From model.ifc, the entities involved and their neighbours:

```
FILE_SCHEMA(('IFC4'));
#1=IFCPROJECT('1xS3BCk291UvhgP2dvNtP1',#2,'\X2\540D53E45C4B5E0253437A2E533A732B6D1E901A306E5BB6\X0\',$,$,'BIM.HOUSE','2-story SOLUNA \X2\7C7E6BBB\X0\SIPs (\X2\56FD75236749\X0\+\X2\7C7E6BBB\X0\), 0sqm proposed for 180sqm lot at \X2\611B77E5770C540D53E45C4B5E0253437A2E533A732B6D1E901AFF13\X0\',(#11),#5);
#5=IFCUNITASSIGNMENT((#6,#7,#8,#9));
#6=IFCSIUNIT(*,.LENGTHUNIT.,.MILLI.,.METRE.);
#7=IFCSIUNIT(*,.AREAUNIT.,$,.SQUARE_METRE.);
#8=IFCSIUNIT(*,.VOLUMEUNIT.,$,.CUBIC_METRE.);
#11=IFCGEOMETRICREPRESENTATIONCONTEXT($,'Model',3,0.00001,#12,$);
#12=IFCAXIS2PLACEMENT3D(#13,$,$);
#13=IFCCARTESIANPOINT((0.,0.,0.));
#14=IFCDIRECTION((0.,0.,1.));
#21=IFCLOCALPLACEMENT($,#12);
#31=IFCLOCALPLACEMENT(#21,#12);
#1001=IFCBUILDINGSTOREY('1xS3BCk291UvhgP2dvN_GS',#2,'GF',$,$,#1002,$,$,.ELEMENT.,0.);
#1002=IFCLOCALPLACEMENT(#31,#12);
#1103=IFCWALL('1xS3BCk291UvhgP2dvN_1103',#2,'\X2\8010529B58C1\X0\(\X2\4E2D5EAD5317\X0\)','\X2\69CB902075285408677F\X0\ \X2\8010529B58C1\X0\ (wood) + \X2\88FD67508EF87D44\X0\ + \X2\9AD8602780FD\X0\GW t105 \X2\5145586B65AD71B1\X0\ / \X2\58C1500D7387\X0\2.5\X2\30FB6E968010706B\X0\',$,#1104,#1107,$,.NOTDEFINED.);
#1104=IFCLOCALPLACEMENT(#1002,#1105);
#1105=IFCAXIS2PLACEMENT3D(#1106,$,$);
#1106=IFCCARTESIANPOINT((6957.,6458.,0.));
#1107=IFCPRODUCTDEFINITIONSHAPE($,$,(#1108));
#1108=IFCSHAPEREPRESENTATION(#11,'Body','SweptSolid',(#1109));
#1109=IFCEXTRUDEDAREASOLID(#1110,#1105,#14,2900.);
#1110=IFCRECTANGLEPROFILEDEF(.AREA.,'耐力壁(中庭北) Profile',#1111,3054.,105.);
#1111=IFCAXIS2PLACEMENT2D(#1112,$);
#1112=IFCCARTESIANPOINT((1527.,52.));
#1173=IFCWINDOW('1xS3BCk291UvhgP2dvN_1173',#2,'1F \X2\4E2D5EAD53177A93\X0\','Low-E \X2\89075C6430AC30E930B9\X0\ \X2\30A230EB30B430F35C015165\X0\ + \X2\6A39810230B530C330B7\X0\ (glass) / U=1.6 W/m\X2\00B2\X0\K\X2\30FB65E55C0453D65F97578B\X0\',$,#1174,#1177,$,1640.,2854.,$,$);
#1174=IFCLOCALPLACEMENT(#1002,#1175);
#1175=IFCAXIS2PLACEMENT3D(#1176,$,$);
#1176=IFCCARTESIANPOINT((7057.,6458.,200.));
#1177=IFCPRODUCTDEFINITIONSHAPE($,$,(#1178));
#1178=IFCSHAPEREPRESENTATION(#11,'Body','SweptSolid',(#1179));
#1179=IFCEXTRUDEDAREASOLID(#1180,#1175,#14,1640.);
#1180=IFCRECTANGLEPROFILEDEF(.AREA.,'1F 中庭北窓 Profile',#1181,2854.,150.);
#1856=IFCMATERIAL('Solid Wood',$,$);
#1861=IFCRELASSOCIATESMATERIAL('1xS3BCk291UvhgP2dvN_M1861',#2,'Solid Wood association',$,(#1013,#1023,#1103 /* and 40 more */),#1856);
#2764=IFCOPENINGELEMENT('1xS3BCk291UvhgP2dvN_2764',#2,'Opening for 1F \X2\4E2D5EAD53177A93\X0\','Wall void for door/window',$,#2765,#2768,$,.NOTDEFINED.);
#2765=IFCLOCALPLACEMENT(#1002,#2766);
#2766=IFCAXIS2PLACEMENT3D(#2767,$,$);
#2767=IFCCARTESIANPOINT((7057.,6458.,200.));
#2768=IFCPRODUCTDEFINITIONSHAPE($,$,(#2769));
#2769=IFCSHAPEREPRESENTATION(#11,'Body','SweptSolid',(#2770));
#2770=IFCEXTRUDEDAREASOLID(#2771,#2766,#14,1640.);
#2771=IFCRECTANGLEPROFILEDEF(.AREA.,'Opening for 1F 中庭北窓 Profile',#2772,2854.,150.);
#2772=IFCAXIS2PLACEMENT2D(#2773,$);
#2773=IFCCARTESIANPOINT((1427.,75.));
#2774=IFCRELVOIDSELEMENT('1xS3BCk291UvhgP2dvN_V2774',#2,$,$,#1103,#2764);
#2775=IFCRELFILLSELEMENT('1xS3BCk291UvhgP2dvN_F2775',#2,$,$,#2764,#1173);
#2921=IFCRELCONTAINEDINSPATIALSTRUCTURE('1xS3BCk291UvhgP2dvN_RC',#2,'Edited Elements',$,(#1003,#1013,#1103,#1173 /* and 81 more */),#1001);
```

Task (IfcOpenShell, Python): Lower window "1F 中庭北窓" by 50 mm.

```python
import numpy as np
import ifcopenshell
import ifcopenshell.api.geometry
import ifcopenshell.util.placement
import ifcopenshell.util.unit

model = ifcopenshell.open("model.ifc")
unit_scale = ifcopenshell.util.unit.calculate_unit_scale(model)

window = model.by_guid("1xS3BCk291UvhgP2dvN_1173")
opening = window.FillsVoids[0].RelatingOpeningElement
dz = -0.05 / unit_scale

shift = np.array([0.0, 0.0, dz])
# The window is not placed relative to its opening, so move both.
for product in (opening, window):
    matrix = ifcopenshell.util.placement.get_local_placement(product.ObjectPlacement)
    matrix[:3, 3] += shift
    ifcopenshell.api.geometry.edit_object_placement(model, product=product, matrix=matrix, is_si=False)

print(f"moved by {dz * unit_scale:+.3f} m")

model.write("model_v2.ifc")
```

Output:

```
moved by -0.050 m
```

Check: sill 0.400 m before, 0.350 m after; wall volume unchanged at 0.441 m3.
